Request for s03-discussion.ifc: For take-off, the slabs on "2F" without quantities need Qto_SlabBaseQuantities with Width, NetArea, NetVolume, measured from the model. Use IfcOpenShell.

First a look at what the model holds.

```python
import ifcopenshell
import ifcopenshell.util.element
import ifcopenshell.util.unit

model = ifcopenshell.open("s03-discussion.ifc")
print(model.schema)
for unit_type in ("LENGTHUNIT", "AREAUNIT", "VOLUMEUNIT"):
    print(unit_type, ifcopenshell.util.unit.calculate_unit_scale(model, unit_type))
storey = next(s for s in model.by_type("IfcBuildingStorey") if s.Name == "2F")
slabs = [e for e in ifcopenshell.util.element.get_decomposition(storey) if e.is_a("IfcSlab")]
for e in sorted(slabs, key=lambda e: e.id()):
    print(e.id(), e.is_a(), e.Name, list(ifcopenshell.util.element.get_psets(e, qtos_only=True)), sep=" | ")
```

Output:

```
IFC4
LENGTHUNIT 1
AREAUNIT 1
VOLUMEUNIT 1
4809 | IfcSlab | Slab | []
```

```python
import ifcopenshell
import ifcopenshell.api.pset
import ifcopenshell.geom
import ifcopenshell.util.element
import ifcopenshell.util.shape
import ifcopenshell.util.unit

model = ifcopenshell.open("s03-discussion.ifc")
unit_scale = ifcopenshell.util.unit.calculate_unit_scale(model)
area_scale = ifcopenshell.util.unit.calculate_unit_scale(model, "AREAUNIT")
volume_scale = ifcopenshell.util.unit.calculate_unit_scale(model, "VOLUMEUNIT")
settings = ifcopenshell.geom.settings()

storey = next(s for s in model.by_type("IfcBuildingStorey") if s.Name == "2F")
slabs = [e for e in ifcopenshell.util.element.get_decomposition(storey) if e.is_a("IfcSlab")]

for e in sorted(slabs, key=lambda e: e.id()):
    if ifcopenshell.util.element.get_psets(e, qtos_only=True, should_inherit=False):
        continue
    # Geometry comes back in metres, in the element's own axes.
    shape = ifcopenshell.geom.create_shape(settings, e)
    values = {
        "Width": ifcopenshell.util.shape.get_z(shape.geometry) / unit_scale,
        "NetArea": ifcopenshell.util.shape.get_footprint_area(shape.geometry) / area_scale,
        "NetVolume": ifcopenshell.util.shape.get_volume(shape.geometry) / volume_scale,
    }
    qto = ifcopenshell.api.pset.add_qto(model, product=e, name="Qto_SlabBaseQuantities")
    ifcopenshell.api.pset.edit_qto(model, qto=qto, properties=values)
    print(e.id(), {k: round(v, 3) for k, v in values.items()})

model.write("s03-discussion-out.ifc")
```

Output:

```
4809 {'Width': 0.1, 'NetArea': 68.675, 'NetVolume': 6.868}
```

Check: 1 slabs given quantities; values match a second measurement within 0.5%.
